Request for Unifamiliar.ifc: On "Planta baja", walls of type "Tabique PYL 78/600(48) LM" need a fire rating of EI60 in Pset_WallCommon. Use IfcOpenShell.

First a look at what the model holds.

```python
import ifcopenshell
import ifcopenshell.util.element

model = ifcopenshell.open("Unifamiliar.ifc")
print(model.schema)
storey = next(s for s in model.by_type("IfcBuildingStorey") if s.Name == "Planta baja")
walls = [e for e in ifcopenshell.util.element.get_decomposition(storey) if e.is_a("IfcWall")]
seen = {}
for e in walls:
    element_type = ifcopenshell.util.element.get_type(e)
    key = (element_type.Name if element_type != e and element_type else None, ifcopenshell.util.element.get_pset(e, "Pset_WallCommon", "FireRating"))
    seen[key] = seen.get(key, 0) + 1
for (name, value), count in sorted(seen.items(), key=str):
    print(count, "x", name, "|", value)
```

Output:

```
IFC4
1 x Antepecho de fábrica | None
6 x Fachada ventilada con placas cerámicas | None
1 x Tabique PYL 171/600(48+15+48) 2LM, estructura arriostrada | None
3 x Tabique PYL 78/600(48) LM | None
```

```python
import ifcopenshell
import ifcopenshell.api.pset
import ifcopenshell.util.element

model = ifcopenshell.open("Unifamiliar.ifc")

storey = next(s for s in model.by_type("IfcBuildingStorey") if s.Name == "Planta baja")
walls = [e for e in ifcopenshell.util.element.get_decomposition(storey) if e.is_a("IfcWall")]

count = 0
for e in walls:
    element_type = ifcopenshell.util.element.get_type(e)
    if element_type in (None, e) or element_type.Name != "Tabique PYL 78/600(48) LM":
        continue
    # add_pset returns the element's existing set when there is one.
    pset = ifcopenshell.api.pset.add_pset(model, product=e, name="Pset_WallCommon")
    ifcopenshell.api.pset.edit_pset(model, pset=pset, properties={"FireRating": "EI60"})
    count += 1

print(count, "walls updated")

model.write("Unifamiliar-out.ifc")
```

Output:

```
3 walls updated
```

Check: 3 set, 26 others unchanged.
